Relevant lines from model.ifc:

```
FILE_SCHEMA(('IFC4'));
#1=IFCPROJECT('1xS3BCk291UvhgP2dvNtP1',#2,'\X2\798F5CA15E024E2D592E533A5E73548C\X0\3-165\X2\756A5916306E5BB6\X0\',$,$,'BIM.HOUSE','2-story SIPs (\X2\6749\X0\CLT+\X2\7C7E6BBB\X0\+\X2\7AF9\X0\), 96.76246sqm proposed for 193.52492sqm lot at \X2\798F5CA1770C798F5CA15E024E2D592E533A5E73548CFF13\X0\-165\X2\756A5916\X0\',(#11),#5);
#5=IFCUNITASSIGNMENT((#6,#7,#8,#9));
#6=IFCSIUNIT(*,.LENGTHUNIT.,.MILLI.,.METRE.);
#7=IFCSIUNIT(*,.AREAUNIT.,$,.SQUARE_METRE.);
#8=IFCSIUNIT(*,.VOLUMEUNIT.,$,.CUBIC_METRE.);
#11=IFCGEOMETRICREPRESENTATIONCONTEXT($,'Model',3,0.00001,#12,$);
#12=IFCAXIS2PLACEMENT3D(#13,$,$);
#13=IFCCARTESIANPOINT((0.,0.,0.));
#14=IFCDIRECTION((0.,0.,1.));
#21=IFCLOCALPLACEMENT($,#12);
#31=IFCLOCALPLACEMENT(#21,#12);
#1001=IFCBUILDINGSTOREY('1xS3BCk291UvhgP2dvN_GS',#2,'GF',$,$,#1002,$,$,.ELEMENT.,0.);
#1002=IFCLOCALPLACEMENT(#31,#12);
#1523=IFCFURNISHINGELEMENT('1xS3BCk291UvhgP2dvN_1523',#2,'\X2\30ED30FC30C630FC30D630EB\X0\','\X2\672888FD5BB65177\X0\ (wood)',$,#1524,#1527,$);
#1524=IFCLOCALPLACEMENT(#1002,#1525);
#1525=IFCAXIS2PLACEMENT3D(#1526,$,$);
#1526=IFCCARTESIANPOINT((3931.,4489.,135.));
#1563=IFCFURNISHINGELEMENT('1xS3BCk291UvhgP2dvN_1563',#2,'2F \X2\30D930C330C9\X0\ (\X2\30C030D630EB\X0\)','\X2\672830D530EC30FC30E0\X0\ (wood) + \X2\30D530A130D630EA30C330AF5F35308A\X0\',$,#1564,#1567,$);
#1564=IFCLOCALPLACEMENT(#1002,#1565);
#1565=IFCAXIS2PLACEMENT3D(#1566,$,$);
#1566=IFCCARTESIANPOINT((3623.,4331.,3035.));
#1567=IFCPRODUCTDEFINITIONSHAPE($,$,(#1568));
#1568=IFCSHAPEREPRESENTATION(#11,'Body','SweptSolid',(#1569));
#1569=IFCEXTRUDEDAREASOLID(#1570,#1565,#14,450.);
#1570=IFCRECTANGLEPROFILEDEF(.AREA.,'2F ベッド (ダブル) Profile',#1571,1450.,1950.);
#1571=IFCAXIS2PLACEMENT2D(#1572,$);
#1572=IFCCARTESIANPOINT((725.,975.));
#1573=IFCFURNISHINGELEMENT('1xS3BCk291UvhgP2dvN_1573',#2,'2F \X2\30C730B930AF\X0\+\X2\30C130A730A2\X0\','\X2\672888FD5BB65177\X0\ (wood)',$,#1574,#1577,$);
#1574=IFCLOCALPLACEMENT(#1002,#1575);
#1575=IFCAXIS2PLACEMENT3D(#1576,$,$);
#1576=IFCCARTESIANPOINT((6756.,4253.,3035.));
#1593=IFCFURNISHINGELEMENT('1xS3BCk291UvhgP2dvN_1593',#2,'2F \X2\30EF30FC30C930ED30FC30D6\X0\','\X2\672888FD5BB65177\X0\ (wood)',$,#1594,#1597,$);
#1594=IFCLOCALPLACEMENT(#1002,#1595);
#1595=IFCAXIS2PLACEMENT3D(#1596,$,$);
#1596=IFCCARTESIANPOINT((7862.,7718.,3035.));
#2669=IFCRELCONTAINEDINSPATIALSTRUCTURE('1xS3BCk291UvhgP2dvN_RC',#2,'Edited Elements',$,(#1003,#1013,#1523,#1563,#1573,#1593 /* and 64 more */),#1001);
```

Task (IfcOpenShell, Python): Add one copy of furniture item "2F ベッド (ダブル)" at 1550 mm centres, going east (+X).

```python
import numpy as np
import ifcopenshell
import ifcopenshell.api.geometry
import ifcopenshell.api.root
import ifcopenshell.util.element
import ifcopenshell.util.placement

model = ifcopenshell.open("model.ifc")


def reuse_history(source, copy):
    """copy_class also copies each property set's owner history, people and application; keep the originals."""
    for rel in copy.IsDefinedBy:
        if rel.is_a("IfcRelDefinesByProperties") and (history := rel.RelatingPropertyDefinition.OwnerHistory):
            rel.RelatingPropertyDefinition.OwnerHistory = source.OwnerHistory
            ifcopenshell.util.element.remove_deep2(model, history)


source = model.by_guid("1xS3BCk291UvhgP2dvN_1563")
base = ifcopenshell.util.placement.get_local_placement(source.ObjectPlacement)
step = np.array([1.0, 0.0, 0.0]) * 1550.0

for i in range(1, 2):
    copy = ifcopenshell.api.root.copy_class(model, product=source)
    copy.Representation = ifcopenshell.util.element.copy_deep(
        model, source.Representation, exclude=["IfcGeometricRepresentationContext", "IfcRepresentationMap"]
    )
    reuse_history(source, copy)
    matrix = base.copy()
    matrix[:3, 3] += i * step
    print("added at", matrix[:3, 3].round(3) + 0.0)
    ifcopenshell.api.geometry.edit_object_placement(model, product=copy, matrix=matrix, is_si=False)

model.write("model_updated.ifc")
```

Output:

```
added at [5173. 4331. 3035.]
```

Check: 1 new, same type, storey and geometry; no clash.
